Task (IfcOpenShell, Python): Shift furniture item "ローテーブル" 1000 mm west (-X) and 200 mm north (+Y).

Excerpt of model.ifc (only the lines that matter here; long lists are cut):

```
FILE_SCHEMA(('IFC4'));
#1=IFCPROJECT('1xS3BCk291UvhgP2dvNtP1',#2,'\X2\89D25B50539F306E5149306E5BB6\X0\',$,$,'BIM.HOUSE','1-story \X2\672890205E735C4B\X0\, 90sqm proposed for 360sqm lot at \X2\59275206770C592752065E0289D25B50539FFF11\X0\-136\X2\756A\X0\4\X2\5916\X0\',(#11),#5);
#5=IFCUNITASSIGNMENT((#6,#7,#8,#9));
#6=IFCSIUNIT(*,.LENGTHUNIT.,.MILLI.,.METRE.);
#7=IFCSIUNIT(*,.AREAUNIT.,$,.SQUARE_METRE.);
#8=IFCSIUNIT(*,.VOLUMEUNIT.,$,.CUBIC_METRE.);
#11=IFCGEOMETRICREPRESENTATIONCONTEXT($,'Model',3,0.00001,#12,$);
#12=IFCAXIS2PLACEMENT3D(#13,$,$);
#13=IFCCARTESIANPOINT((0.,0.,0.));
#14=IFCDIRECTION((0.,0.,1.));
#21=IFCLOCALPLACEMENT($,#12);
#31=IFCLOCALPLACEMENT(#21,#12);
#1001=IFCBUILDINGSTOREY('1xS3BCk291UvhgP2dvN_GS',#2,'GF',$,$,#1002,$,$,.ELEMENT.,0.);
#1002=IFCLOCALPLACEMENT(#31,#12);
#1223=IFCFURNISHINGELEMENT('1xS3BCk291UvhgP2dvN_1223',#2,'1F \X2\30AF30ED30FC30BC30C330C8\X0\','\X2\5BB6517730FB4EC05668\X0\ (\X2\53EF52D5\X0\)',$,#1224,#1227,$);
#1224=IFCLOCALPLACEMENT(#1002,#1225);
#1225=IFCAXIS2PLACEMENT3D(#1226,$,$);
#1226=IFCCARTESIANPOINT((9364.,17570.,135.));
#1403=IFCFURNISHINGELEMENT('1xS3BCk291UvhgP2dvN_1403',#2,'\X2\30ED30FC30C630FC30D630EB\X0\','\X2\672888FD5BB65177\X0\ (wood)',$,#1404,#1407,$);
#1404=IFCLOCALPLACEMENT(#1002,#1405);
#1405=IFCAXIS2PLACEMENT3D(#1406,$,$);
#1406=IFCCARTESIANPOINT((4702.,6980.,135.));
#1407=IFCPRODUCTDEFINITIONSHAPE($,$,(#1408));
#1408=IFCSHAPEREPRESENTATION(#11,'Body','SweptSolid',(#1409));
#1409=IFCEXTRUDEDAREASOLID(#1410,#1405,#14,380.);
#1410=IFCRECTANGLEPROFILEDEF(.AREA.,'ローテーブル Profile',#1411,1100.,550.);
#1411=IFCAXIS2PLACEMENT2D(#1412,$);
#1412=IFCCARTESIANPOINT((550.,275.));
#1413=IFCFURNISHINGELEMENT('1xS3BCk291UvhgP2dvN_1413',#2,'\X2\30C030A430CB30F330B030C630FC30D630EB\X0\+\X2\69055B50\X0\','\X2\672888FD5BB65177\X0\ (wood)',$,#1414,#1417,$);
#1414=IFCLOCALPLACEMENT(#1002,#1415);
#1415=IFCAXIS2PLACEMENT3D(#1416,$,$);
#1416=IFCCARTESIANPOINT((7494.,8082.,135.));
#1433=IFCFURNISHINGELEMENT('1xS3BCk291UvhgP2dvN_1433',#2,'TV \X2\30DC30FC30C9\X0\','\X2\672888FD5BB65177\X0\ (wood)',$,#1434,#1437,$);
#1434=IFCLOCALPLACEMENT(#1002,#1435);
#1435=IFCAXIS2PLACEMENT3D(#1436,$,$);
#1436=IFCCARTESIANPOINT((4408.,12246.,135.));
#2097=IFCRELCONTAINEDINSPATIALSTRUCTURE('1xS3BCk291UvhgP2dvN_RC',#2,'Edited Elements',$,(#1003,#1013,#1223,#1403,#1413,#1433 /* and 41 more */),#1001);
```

```python
import ifcopenshell
import ifcopenshell.api.geometry
import ifcopenshell.util.placement
import ifcopenshell.util.unit

model = ifcopenshell.open("model.ifc")
unit_scale = ifcopenshell.util.unit.calculate_unit_scale(model)

item = model.by_guid("1xS3BCk291UvhgP2dvN_1403")
matrix = ifcopenshell.util.placement.get_local_placement(item.ObjectPlacement)
matrix[0, 3] -= 1 / unit_scale
matrix[1, 3] += 0.2 / unit_scale
ifcopenshell.api.geometry.edit_object_placement(model, product=item, matrix=matrix, is_si=False)

print(ifcopenshell.util.placement.get_local_placement(item.ObjectPlacement).round(3) + 0.0)

model.write("model_v2.ifc")
```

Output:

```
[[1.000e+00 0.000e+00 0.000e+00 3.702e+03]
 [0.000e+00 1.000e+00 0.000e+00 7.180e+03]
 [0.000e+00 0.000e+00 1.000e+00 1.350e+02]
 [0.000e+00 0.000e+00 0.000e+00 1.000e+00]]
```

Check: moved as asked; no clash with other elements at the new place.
